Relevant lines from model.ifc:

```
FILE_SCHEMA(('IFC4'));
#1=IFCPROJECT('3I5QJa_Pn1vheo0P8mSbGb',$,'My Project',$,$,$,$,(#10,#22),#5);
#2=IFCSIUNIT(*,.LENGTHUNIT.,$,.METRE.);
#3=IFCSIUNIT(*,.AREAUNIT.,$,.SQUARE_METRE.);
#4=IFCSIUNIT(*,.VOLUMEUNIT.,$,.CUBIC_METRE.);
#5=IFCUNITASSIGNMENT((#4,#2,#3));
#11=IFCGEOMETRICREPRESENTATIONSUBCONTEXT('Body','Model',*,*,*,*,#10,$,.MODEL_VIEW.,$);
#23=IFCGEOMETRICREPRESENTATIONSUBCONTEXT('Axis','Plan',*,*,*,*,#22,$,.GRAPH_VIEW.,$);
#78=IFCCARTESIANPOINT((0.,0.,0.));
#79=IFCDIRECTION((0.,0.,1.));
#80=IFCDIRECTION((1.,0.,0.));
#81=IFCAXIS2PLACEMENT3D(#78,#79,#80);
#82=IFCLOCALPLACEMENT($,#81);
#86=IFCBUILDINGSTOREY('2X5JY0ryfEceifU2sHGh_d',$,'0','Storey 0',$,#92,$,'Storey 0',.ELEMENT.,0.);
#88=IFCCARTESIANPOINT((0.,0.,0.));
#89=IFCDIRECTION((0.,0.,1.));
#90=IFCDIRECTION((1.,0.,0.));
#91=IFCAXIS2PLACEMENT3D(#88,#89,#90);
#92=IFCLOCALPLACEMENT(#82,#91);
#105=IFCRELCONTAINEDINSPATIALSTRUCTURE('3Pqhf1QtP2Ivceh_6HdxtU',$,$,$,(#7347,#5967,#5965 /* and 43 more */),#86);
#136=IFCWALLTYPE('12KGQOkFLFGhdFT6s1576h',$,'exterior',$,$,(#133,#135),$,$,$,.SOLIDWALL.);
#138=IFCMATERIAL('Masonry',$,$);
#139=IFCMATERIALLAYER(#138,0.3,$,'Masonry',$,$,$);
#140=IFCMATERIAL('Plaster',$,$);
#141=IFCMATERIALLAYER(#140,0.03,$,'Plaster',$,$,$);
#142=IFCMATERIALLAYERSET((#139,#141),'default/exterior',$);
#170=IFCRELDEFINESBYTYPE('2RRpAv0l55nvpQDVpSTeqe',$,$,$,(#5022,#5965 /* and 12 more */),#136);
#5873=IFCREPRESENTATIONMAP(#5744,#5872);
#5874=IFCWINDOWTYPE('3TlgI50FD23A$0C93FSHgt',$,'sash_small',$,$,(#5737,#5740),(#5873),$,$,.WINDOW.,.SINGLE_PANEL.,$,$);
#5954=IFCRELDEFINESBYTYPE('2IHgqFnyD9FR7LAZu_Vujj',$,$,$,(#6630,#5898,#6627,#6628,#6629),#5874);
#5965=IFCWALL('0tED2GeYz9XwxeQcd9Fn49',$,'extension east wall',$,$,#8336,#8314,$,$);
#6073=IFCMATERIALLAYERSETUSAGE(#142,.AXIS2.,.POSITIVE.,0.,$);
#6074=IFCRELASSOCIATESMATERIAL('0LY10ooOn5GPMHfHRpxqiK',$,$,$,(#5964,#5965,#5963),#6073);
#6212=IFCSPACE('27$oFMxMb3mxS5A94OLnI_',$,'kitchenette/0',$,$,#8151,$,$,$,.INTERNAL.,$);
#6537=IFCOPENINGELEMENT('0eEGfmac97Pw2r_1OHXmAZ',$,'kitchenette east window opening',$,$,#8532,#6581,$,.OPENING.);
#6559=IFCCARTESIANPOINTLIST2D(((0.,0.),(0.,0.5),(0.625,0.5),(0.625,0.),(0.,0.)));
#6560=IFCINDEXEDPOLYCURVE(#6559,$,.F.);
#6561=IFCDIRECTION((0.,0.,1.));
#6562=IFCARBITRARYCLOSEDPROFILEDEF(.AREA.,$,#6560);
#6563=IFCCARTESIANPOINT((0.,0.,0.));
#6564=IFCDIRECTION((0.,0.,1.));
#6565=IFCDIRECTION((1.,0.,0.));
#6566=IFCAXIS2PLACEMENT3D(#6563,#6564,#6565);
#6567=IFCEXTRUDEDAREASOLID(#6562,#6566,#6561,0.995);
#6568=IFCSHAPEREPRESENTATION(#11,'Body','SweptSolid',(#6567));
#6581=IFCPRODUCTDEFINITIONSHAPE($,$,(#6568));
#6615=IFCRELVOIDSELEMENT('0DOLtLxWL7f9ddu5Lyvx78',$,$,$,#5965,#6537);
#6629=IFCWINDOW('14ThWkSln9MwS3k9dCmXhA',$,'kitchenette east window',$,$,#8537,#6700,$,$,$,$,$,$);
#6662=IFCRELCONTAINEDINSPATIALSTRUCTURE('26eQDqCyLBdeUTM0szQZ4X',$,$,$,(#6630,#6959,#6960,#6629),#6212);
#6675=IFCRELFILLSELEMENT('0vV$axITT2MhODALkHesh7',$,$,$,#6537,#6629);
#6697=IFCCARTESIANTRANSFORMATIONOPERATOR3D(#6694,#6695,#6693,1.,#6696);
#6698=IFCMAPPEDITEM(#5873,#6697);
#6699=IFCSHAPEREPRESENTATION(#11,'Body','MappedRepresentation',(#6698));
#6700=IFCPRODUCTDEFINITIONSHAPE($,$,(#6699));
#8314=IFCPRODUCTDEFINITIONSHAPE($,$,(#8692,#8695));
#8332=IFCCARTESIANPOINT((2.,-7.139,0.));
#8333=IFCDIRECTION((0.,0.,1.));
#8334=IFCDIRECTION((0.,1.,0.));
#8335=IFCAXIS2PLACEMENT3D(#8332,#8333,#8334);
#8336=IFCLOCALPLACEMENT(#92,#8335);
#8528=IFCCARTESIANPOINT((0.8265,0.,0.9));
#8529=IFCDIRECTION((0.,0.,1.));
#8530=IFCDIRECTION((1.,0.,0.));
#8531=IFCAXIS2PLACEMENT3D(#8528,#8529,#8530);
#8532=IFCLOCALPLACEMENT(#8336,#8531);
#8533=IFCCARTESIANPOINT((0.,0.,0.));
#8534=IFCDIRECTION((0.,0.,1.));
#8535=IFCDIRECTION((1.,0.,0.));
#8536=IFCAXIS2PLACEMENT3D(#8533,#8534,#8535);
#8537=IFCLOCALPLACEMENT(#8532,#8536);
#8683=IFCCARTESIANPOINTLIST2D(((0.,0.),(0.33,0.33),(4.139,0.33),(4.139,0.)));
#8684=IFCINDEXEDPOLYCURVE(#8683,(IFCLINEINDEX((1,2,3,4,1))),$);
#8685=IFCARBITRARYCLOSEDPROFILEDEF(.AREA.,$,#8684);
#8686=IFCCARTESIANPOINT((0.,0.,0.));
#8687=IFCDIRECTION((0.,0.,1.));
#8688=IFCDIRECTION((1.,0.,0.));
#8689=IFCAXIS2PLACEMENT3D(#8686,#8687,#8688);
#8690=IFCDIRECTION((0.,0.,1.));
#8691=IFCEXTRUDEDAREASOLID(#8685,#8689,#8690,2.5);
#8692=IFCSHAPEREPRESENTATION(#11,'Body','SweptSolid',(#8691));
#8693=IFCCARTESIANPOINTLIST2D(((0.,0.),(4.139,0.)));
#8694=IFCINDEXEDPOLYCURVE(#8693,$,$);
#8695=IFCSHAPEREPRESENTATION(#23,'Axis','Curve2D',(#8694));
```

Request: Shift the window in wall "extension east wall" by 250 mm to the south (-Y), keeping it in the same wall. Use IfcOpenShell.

```python
import ifcopenshell
import ifcopenshell.api.geometry
import ifcopenshell.util.placement
import ifcopenshell.util.unit

model = ifcopenshell.open("model.ifc")
unit_scale = ifcopenshell.util.unit.calculate_unit_scale(model)

window = model.by_guid("14ThWkSln9MwS3k9dCmXhA")
opening = window.FillsVoids[0].RelatingOpeningElement
wall = opening.VoidsElements[0].RelatingBuildingElement

wall_matrix = ifcopenshell.util.placement.get_local_placement(wall.ObjectPlacement)
shift = wall_matrix[:3, 0] * -0.25 / unit_scale
before = ifcopenshell.util.placement.get_local_placement(window.ObjectPlacement)[:3, 3].copy()

# The window is placed relative to its opening, so it follows when the opening moves.
matrix = ifcopenshell.util.placement.get_local_placement(opening.ObjectPlacement)
matrix[:3, 3] += shift
ifcopenshell.api.geometry.edit_object_placement(
    model, product=opening, matrix=matrix, is_si=False, should_transform_children=True
)

after = ifcopenshell.util.placement.get_local_placement(window.ObjectPlacement)[:3, 3]
print("window moved by", (after - before).round(3) + 0.0)

model.write("model-out.ifc")
```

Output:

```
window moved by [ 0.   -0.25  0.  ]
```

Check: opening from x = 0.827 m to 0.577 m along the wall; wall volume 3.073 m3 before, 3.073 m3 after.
